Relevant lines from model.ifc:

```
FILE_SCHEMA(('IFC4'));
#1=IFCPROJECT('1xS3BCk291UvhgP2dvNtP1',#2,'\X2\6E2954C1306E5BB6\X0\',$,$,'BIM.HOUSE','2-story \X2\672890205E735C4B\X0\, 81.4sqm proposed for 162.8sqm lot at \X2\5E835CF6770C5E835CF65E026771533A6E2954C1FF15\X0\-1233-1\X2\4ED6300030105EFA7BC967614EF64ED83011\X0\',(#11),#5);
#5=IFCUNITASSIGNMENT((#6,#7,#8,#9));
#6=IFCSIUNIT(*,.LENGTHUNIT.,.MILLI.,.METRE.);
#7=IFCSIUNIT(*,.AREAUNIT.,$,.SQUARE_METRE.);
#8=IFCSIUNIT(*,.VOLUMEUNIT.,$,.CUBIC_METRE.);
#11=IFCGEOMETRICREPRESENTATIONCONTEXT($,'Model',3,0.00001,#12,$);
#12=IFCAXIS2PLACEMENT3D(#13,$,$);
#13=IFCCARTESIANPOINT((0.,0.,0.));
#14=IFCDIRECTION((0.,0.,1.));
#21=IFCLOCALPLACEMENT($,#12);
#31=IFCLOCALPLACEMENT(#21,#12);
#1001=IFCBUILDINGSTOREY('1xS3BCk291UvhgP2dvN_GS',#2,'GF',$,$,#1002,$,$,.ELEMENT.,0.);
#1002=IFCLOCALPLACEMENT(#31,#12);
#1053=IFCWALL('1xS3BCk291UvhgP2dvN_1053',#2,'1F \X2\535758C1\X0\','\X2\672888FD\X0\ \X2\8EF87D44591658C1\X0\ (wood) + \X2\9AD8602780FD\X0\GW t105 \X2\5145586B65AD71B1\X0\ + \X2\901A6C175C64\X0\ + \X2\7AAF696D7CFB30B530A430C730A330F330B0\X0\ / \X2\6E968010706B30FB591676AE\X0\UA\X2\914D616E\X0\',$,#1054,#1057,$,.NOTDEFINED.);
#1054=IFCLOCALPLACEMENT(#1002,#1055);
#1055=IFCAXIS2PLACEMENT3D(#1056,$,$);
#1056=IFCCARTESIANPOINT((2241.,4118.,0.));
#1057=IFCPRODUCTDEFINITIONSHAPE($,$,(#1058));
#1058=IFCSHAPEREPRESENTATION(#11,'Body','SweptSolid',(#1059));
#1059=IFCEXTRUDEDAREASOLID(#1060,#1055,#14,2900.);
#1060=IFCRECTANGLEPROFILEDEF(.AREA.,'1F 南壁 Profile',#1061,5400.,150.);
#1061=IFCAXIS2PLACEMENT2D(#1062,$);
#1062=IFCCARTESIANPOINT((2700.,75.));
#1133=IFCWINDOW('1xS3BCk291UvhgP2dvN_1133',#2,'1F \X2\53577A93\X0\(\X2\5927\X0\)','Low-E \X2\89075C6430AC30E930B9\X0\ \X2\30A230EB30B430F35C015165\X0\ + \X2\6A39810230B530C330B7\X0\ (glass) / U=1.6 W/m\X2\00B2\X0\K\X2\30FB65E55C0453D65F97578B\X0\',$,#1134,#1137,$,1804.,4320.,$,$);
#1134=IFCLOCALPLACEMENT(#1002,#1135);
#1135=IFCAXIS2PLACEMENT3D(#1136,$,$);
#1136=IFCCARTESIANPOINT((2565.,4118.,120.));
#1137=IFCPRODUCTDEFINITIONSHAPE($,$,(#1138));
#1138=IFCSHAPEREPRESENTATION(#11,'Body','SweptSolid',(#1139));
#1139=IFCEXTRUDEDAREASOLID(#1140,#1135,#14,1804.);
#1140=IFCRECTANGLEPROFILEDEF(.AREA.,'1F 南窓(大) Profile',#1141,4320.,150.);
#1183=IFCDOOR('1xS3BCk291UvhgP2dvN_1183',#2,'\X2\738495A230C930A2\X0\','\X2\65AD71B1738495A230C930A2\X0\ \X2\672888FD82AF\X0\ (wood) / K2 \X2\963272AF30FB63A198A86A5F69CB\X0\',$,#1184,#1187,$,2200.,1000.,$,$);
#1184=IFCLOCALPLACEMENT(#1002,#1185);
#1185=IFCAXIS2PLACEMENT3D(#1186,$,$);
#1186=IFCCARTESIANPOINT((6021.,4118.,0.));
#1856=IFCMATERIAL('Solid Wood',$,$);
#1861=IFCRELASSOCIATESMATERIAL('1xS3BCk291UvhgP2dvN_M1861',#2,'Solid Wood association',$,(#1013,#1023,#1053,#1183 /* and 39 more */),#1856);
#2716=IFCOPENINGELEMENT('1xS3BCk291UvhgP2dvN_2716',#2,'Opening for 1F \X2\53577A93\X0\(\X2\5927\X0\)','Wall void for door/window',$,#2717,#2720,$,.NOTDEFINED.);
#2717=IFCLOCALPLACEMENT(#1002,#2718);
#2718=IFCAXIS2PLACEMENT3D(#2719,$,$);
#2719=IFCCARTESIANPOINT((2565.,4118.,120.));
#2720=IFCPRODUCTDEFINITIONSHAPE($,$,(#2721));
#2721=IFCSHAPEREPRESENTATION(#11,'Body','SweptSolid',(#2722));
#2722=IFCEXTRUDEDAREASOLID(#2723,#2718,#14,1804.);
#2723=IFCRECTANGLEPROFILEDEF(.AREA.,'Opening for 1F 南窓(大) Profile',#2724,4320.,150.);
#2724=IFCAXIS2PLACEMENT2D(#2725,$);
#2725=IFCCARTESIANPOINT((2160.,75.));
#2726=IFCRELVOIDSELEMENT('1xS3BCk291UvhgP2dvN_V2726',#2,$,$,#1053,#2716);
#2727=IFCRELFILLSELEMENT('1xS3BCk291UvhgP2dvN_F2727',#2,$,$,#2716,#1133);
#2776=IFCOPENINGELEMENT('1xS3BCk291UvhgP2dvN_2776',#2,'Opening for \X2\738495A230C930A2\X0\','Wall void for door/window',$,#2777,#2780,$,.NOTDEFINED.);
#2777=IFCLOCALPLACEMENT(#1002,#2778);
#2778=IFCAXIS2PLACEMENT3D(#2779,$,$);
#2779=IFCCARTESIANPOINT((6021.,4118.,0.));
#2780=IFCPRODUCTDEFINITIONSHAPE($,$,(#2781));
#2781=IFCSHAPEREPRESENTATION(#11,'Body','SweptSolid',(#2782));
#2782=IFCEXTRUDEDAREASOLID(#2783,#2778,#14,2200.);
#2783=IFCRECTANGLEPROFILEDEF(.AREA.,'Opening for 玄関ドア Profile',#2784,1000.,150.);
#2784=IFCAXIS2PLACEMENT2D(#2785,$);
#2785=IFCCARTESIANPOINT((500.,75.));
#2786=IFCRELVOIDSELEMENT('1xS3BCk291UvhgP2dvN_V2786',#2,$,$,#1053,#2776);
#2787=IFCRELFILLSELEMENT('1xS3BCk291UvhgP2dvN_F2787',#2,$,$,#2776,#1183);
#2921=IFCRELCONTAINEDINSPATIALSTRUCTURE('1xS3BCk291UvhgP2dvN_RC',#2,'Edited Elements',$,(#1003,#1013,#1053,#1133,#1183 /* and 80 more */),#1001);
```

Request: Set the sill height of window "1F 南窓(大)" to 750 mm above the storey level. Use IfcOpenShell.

```python
import numpy as np
import ifcopenshell
import ifcopenshell.api.geometry
import ifcopenshell.geom
import ifcopenshell.util.element
import ifcopenshell.util.placement
import ifcopenshell.util.shape
import ifcopenshell.util.unit

model = ifcopenshell.open("model.ifc")
unit_scale = ifcopenshell.util.unit.calculate_unit_scale(model)

window = model.by_guid("1xS3BCk291UvhgP2dvN_1133")
opening = window.FillsVoids[0].RelatingOpeningElement
storey = ifcopenshell.util.element.get_container(window, ifc_class="IfcBuildingStorey")
level = ifcopenshell.util.placement.get_local_placement(storey.ObjectPlacement)[2, 3]

# The opening's origin need not be at the sill, so measure its lowest point.
shape = ifcopenshell.geom.create_shape(ifcopenshell.geom.settings(), opening)
bottom = ifcopenshell.util.shape.get_shape_bottom_elevation(shape, shape.geometry) / unit_scale
dz = level + 0.75 / unit_scale - bottom

shift = np.array([0.0, 0.0, dz])
# The window is not placed relative to its opening, so move both.
for product in (opening, window):
    matrix = ifcopenshell.util.placement.get_local_placement(product.ObjectPlacement)
    matrix[:3, 3] += shift
    ifcopenshell.api.geometry.edit_object_placement(model, product=product, matrix=matrix, is_si=False)

print(f"moved by {dz * unit_scale:+.3f} m")

model.write("model_rev.ifc")
```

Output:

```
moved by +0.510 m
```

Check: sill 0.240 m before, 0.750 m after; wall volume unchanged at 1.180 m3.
